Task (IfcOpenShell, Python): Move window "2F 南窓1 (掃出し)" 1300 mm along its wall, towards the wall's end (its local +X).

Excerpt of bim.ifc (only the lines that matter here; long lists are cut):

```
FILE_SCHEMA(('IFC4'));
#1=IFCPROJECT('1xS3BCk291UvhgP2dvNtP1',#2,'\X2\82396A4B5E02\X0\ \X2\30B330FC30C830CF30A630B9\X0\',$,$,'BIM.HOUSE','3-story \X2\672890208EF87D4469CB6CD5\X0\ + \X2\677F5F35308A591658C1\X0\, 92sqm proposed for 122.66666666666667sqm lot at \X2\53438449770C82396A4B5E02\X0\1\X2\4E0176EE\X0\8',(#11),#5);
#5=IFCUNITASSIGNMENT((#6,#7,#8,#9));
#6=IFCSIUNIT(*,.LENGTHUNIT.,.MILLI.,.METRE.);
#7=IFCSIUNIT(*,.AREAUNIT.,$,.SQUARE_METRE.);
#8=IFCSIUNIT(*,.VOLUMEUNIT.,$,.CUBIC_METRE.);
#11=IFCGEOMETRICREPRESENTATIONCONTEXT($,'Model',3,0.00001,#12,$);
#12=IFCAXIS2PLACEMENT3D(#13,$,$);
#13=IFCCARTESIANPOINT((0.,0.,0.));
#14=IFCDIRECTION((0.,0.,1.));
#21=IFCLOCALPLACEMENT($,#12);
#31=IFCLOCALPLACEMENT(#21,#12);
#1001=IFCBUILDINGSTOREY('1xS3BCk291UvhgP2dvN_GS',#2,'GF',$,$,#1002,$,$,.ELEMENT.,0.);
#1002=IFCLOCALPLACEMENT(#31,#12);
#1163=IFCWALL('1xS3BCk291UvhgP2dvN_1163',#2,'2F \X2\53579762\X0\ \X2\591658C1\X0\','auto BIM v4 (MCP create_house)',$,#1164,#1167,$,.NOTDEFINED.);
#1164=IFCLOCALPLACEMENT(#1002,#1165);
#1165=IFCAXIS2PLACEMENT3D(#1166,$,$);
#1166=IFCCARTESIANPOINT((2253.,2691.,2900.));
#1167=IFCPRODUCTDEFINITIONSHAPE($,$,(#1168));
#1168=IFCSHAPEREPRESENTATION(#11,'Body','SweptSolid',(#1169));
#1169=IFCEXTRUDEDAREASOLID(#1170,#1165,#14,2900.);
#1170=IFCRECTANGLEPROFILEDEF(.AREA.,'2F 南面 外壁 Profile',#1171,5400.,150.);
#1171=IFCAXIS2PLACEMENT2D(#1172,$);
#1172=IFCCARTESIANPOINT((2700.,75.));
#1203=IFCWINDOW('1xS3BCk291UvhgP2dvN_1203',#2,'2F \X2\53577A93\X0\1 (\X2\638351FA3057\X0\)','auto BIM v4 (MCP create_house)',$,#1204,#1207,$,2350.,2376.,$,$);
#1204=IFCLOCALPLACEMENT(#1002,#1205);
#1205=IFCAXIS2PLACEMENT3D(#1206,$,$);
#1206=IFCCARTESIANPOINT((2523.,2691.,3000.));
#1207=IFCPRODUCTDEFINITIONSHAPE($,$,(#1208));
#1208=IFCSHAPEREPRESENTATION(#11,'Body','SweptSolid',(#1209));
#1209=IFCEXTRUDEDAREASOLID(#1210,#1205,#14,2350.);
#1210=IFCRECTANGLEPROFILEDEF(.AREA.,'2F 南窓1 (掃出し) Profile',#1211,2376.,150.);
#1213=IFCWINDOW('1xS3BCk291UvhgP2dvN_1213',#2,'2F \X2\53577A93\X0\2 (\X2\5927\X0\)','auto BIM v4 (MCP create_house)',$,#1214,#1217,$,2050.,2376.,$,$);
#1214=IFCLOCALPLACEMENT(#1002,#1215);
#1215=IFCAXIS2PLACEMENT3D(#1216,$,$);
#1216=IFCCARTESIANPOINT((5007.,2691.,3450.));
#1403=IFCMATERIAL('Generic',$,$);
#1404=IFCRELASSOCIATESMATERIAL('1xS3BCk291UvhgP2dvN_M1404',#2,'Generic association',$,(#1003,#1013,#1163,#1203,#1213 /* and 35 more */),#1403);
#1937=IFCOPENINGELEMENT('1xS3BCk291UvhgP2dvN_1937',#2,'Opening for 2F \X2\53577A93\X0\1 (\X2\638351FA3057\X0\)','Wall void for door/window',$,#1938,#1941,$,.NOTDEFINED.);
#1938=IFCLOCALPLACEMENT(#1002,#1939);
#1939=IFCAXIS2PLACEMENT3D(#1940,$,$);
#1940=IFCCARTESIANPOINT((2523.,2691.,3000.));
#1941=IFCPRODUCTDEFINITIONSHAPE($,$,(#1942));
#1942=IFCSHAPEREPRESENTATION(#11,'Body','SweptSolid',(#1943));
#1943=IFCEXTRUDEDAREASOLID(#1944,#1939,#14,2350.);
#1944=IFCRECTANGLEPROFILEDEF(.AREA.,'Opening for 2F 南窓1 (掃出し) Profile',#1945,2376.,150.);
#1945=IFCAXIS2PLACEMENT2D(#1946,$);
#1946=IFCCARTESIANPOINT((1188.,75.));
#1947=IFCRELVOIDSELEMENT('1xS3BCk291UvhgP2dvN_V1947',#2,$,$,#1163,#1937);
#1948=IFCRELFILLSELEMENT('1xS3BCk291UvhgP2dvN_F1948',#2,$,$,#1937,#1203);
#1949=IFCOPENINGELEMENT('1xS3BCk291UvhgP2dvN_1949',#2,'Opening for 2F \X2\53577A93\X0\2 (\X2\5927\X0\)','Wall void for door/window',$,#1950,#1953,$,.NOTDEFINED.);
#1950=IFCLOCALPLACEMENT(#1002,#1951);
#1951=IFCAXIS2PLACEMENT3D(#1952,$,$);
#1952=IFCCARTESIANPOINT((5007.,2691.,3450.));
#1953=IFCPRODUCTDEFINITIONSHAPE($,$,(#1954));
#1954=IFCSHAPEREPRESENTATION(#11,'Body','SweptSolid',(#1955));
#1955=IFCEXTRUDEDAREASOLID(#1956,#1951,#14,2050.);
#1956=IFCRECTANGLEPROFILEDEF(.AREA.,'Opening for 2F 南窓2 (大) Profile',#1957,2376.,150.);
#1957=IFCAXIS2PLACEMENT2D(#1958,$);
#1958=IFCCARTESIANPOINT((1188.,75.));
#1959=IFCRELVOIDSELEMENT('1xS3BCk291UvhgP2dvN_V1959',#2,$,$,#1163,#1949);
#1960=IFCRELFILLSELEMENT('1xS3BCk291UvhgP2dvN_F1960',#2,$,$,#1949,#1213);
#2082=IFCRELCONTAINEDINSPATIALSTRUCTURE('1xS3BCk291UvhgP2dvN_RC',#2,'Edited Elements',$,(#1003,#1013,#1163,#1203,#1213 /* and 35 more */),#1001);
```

```python
import ifcopenshell
import ifcopenshell.api.geometry
import ifcopenshell.util.placement
import ifcopenshell.util.unit

model = ifcopenshell.open("bim.ifc")
unit_scale = ifcopenshell.util.unit.calculate_unit_scale(model)

window = model.by_guid("1xS3BCk291UvhgP2dvN_1203")
opening = window.FillsVoids[0].RelatingOpeningElement
wall = opening.VoidsElements[0].RelatingBuildingElement

wall_matrix = ifcopenshell.util.placement.get_local_placement(wall.ObjectPlacement)
shift = wall_matrix[:3, 0] * 1.3 / unit_scale
before = ifcopenshell.util.placement.get_local_placement(window.ObjectPlacement)[:3, 3].copy()

# The window is not placed relative to its opening, so move both.
for product in (opening, window):
    matrix = ifcopenshell.util.placement.get_local_placement(product.ObjectPlacement)
    matrix[:3, 3] += shift
    ifcopenshell.api.geometry.edit_object_placement(model, product=product, matrix=matrix, is_si=False)

after = ifcopenshell.util.placement.get_local_placement(window.ObjectPlacement)[:3, 3]
print("window moved by", (after - before).round(3) + 0.0)

model.write("bim_updated.ifc")
```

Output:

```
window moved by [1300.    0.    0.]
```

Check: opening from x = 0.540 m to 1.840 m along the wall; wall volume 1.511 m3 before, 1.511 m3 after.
